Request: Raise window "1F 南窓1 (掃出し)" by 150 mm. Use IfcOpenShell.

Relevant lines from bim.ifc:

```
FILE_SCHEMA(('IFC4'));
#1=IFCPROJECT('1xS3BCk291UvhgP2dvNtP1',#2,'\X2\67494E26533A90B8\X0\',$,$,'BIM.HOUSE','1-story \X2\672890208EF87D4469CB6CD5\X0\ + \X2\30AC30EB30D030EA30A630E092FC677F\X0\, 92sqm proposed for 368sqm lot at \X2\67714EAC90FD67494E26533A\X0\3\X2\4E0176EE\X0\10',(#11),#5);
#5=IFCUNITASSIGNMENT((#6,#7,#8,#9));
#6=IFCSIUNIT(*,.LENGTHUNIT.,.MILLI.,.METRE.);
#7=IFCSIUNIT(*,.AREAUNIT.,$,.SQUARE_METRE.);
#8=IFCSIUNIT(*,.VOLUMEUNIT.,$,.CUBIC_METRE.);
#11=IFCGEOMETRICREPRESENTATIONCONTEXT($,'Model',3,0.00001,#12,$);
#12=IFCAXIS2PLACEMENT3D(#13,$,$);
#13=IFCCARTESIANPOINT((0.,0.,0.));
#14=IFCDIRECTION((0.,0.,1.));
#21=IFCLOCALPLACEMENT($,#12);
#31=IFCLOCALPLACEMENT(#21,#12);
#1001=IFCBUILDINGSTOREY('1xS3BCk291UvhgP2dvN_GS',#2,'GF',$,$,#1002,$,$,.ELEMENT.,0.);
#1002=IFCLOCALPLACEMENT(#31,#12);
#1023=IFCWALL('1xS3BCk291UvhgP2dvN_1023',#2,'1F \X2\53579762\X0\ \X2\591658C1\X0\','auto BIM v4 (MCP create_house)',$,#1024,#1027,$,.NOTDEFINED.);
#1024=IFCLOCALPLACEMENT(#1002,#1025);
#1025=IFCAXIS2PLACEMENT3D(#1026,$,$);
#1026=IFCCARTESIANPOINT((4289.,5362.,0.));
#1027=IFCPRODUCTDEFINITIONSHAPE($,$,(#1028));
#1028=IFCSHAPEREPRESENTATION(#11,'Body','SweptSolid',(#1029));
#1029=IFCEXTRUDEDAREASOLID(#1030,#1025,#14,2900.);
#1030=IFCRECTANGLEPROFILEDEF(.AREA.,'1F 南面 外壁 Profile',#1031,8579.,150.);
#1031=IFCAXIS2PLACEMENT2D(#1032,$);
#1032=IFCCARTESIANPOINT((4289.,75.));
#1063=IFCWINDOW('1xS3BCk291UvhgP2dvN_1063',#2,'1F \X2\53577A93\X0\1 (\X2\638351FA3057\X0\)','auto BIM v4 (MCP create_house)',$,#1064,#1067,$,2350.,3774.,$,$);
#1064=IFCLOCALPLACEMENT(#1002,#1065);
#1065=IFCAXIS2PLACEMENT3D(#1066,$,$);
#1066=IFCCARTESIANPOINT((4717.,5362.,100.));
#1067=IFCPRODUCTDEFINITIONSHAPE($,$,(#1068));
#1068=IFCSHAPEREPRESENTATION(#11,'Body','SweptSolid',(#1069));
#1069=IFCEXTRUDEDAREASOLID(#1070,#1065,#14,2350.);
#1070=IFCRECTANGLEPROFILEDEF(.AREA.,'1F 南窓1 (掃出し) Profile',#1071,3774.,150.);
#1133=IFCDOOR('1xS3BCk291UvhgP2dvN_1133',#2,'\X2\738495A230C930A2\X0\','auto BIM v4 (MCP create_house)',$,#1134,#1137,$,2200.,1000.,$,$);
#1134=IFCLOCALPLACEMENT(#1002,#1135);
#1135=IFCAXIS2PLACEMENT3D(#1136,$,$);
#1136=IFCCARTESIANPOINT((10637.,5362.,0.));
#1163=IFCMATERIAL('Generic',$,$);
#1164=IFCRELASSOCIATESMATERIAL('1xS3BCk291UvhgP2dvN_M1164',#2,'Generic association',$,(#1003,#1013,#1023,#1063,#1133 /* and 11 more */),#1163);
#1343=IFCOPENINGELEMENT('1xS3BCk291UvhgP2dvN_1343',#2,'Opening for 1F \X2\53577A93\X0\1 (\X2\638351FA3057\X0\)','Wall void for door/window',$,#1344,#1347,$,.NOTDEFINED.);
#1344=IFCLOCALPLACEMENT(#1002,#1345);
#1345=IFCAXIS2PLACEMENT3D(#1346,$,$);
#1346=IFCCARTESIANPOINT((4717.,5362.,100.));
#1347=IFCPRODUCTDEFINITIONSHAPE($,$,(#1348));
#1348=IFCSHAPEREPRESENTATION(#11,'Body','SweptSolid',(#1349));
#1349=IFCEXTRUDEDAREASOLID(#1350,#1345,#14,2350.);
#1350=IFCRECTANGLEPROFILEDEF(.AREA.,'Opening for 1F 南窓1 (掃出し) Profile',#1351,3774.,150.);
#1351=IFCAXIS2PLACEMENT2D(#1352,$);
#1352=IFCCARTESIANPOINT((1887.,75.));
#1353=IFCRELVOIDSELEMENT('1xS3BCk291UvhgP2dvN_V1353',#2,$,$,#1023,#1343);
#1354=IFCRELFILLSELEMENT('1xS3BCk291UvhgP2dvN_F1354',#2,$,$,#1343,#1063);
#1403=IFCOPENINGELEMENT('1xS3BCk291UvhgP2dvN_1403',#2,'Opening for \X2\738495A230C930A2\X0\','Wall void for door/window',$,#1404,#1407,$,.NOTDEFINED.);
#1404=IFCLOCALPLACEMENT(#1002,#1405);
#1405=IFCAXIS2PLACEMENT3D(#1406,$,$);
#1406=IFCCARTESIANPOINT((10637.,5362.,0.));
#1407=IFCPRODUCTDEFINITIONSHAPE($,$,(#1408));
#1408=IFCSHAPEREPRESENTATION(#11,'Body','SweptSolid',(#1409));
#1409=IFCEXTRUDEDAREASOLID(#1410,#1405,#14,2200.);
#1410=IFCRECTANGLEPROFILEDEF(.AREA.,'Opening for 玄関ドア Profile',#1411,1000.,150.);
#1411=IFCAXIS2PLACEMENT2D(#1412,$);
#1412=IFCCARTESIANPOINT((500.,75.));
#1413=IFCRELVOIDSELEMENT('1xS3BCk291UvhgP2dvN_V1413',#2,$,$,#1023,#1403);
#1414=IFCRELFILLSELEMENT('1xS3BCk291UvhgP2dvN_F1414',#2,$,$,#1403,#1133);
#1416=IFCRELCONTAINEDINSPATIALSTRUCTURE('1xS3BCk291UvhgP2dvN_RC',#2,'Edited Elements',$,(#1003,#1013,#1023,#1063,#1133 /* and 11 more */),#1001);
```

```python
import numpy as np
import ifcopenshell
import ifcopenshell.api.geometry
import ifcopenshell.util.placement
import ifcopenshell.util.unit

model = ifcopenshell.open("bim.ifc")
unit_scale = ifcopenshell.util.unit.calculate_unit_scale(model)

window = model.by_id(1063)
opening = window.FillsVoids[0].RelatingOpeningElement
dz = 150.0

shift = np.array([0.0, 0.0, dz])
# The window is not placed relative to its opening, so move both.
for product in (opening, window):
    matrix = ifcopenshell.util.placement.get_local_placement(product.ObjectPlacement)
    matrix[:3, 3] += shift
    ifcopenshell.api.geometry.edit_object_placement(model, product=product, matrix=matrix, is_si=False)

print(f"moved by {dz * unit_scale:+.3f} m")

model.write("bim_v2.ifc")
```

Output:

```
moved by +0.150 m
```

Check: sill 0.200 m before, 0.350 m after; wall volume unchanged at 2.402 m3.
